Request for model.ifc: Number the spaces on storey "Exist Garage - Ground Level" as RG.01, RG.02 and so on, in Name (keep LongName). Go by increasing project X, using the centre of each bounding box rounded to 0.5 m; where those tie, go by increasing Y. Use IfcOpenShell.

First a look at what the model holds.

```python
import ifcopenshell
import ifcopenshell.util.element
import ifcopenshell.util.placement

model = ifcopenshell.open("model.ifc")
print(model.schema)
storey = next(s for s in model.by_type("IfcBuildingStorey") if s.Name == "Exist Garage - Ground Level")
spaces = [e for e in ifcopenshell.util.element.get_decomposition(storey) if e.is_a("IfcSpace")]
for e in sorted(spaces, key=lambda e: e.id()):
    origin = ifcopenshell.util.placement.get_local_placement(e.ObjectPlacement)[:3, 3]
    print(e.id(), e.Name, e.LongName, origin.round(2) + 0.0, sep=" | ")
```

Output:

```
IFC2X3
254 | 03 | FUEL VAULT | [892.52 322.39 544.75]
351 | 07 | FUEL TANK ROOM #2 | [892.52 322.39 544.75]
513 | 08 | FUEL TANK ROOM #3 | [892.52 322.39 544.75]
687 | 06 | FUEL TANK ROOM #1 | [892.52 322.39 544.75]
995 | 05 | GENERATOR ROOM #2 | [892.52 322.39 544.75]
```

```python
import ifcopenshell
import ifcopenshell.geom
import ifcopenshell.util.element
import ifcopenshell.util.shape

model = ifcopenshell.open("model.ifc")
settings = ifcopenshell.geom.settings()
settings.set("use-world-coords", True)


def centre(element):
    shape = ifcopenshell.geom.create_shape(settings, element)
    return ifcopenshell.util.shape.get_bbox_centroid(shape.geometry)


storey = next(s for s in model.by_type("IfcBuildingStorey") if s.Name == "Exist Garage - Ground Level")
spaces = [e for e in ifcopenshell.util.element.get_decomposition(storey) if e.is_a("IfcSpace")]

# Insertion points can sit at a corner or the storey origin, so sort by the geometry (in metres).
centres = {e: centre(e) for e in spaces}
spaces.sort(key=lambda e: (round(centres[e][0] / 0.5), centres[e][1]))

for i, e in enumerate(spaces, start=1):
    number = f"RG.{i:02d}"
    e.Name = number
    print(e.id(), number)

model.write("model_edited.ifc")
```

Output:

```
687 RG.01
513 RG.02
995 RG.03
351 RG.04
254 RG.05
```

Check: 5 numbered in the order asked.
